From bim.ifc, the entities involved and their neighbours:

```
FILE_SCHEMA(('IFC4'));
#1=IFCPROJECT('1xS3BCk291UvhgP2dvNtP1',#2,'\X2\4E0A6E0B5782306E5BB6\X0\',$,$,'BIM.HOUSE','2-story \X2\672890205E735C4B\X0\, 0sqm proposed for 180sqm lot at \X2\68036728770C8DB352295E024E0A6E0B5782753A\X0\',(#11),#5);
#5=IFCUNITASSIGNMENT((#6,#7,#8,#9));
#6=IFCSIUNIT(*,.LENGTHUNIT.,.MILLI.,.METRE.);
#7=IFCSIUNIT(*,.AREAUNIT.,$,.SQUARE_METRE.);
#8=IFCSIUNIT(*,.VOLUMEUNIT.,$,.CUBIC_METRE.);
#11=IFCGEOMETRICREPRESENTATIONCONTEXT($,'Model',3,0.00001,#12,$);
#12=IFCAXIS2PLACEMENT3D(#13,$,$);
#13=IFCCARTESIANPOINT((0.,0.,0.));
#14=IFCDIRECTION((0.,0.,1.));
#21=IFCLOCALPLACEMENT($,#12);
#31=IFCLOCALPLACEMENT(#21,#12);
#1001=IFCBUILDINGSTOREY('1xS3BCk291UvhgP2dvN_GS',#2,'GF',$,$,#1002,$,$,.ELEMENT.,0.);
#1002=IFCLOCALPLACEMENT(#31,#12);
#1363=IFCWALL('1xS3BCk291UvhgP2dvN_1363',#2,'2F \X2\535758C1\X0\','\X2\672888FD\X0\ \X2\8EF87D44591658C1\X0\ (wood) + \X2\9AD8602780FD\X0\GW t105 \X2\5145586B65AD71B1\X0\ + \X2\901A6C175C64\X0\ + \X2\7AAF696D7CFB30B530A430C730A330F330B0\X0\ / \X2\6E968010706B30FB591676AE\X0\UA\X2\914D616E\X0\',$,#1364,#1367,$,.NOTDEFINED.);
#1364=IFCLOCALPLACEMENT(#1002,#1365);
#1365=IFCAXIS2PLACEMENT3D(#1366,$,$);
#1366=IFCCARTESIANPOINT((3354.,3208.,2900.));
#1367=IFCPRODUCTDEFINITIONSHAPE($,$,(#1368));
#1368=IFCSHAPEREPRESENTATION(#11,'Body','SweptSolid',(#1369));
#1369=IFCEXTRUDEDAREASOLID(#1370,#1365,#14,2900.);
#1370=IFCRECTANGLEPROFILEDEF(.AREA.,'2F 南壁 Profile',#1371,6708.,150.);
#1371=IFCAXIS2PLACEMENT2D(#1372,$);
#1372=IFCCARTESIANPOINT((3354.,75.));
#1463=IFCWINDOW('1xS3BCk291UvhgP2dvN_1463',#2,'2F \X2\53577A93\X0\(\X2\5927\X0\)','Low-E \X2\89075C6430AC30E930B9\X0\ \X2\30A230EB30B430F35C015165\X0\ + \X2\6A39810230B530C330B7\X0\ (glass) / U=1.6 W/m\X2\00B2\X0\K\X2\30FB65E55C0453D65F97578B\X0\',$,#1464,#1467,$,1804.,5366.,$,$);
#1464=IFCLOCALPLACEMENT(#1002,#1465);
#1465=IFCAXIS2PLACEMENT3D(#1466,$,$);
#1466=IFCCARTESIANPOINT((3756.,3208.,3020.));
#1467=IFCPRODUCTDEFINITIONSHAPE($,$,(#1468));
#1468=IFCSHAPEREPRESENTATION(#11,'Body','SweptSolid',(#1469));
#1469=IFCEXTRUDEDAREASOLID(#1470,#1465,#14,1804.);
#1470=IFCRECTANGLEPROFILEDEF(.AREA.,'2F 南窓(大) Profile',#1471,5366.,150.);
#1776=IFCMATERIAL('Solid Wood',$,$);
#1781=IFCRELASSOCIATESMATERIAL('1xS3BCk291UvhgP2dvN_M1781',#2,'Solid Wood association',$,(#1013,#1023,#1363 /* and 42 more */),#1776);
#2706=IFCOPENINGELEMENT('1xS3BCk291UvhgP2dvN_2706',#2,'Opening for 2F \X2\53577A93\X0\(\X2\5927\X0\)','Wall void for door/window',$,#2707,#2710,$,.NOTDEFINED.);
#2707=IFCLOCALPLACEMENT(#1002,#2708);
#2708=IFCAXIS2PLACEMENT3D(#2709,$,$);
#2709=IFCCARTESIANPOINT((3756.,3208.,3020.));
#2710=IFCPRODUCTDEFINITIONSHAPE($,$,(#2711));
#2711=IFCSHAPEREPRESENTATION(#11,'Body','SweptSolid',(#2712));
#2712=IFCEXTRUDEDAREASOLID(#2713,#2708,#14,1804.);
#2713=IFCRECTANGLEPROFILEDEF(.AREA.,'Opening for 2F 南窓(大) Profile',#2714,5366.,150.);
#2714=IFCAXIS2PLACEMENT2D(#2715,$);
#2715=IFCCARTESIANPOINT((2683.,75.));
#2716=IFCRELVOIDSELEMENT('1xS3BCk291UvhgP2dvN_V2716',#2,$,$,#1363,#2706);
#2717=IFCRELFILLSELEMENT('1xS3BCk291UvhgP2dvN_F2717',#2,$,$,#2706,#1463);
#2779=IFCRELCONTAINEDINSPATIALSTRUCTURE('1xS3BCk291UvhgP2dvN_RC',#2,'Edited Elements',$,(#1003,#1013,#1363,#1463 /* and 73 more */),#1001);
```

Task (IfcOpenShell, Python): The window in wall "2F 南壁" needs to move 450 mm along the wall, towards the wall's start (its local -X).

```python
import ifcopenshell
import ifcopenshell.api.geometry
import ifcopenshell.util.placement

model = ifcopenshell.open("bim.ifc")

window = model.by_guid("1xS3BCk291UvhgP2dvN_1463")
opening = window.FillsVoids[0].RelatingOpeningElement
wall = opening.VoidsElements[0].RelatingBuildingElement

wall_matrix = ifcopenshell.util.placement.get_local_placement(wall.ObjectPlacement)
shift = wall_matrix[:3, 0] * -450.0
before = ifcopenshell.util.placement.get_local_placement(window.ObjectPlacement)[:3, 3].copy()

# The window is not placed relative to its opening, so move both.
for product in (opening, window):
    matrix = ifcopenshell.util.placement.get_local_placement(product.ObjectPlacement)
    matrix[:3, 3] += shift
    ifcopenshell.api.geometry.edit_object_placement(model, product=product, matrix=matrix, is_si=False)

after = ifcopenshell.util.placement.get_local_placement(window.ObjectPlacement)[:3, 3]
print("window moved by", (after - before).round(3) + 0.0)

model.write("bim_rev.ifc")
```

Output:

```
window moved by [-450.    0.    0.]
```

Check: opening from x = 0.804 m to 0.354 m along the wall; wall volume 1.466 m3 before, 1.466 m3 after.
